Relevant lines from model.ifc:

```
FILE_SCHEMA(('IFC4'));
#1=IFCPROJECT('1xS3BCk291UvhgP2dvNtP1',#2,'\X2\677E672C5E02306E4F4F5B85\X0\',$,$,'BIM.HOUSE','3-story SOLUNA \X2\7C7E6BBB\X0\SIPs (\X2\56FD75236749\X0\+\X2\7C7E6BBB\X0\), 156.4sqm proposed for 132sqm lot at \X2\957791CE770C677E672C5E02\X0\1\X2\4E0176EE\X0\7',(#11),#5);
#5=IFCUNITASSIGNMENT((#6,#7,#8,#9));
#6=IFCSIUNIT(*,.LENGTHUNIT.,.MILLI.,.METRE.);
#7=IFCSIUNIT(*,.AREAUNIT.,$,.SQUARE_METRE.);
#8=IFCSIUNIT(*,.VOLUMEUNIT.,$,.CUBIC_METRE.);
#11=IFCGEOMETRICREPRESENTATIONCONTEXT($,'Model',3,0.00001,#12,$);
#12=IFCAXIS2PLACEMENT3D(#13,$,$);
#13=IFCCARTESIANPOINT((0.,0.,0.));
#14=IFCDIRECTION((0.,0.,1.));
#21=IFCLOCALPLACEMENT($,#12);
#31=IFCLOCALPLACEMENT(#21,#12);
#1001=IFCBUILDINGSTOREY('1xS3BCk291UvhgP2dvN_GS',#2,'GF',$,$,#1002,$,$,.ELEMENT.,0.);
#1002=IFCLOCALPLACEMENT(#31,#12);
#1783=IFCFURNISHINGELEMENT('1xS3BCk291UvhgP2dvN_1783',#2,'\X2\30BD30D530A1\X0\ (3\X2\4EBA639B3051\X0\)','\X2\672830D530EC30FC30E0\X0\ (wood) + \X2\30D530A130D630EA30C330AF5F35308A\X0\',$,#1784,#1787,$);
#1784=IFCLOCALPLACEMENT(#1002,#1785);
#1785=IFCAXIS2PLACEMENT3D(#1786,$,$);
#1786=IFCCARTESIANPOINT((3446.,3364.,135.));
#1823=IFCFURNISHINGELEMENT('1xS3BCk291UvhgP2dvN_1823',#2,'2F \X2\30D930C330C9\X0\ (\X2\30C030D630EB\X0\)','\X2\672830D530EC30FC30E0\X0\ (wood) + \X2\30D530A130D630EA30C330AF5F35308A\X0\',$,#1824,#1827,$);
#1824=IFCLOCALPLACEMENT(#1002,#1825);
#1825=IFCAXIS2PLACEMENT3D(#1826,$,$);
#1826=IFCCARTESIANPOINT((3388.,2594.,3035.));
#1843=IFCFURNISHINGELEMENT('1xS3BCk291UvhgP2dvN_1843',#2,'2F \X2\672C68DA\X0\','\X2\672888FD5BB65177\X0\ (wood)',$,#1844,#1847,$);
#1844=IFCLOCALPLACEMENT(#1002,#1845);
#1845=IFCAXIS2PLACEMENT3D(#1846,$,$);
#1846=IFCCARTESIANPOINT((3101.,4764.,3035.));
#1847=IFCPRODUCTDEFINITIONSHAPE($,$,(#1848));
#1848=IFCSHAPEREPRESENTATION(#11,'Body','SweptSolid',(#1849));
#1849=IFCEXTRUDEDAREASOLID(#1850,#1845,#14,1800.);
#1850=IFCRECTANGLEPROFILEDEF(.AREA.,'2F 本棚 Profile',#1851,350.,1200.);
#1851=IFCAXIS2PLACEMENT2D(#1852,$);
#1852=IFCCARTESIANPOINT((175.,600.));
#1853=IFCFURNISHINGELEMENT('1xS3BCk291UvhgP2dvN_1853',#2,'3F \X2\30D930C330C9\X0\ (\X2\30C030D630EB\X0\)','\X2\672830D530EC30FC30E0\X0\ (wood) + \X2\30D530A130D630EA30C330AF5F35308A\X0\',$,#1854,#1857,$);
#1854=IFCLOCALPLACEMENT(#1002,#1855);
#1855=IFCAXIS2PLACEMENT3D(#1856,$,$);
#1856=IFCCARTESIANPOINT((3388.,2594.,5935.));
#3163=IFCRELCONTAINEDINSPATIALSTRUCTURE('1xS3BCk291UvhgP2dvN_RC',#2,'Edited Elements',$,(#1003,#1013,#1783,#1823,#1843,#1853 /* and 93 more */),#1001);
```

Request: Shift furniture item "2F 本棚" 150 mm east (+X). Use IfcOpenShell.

```python
import ifcopenshell
import ifcopenshell.api.geometry
import ifcopenshell.util.placement
import ifcopenshell.util.unit

model = ifcopenshell.open("model.ifc")
unit_scale = ifcopenshell.util.unit.calculate_unit_scale(model)

item = model.by_id(1843)
matrix = ifcopenshell.util.placement.get_local_placement(item.ObjectPlacement)
matrix[0, 3] += 0.15 / unit_scale
ifcopenshell.api.geometry.edit_object_placement(model, product=item, matrix=matrix, is_si=False)

print(ifcopenshell.util.placement.get_local_placement(item.ObjectPlacement).round(3) + 0.0)

model.write("model_updated.ifc")
```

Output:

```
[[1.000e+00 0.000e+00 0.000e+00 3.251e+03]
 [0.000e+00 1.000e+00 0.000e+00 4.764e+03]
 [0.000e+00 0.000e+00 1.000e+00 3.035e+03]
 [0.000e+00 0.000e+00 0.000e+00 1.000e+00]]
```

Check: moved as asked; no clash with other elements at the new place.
